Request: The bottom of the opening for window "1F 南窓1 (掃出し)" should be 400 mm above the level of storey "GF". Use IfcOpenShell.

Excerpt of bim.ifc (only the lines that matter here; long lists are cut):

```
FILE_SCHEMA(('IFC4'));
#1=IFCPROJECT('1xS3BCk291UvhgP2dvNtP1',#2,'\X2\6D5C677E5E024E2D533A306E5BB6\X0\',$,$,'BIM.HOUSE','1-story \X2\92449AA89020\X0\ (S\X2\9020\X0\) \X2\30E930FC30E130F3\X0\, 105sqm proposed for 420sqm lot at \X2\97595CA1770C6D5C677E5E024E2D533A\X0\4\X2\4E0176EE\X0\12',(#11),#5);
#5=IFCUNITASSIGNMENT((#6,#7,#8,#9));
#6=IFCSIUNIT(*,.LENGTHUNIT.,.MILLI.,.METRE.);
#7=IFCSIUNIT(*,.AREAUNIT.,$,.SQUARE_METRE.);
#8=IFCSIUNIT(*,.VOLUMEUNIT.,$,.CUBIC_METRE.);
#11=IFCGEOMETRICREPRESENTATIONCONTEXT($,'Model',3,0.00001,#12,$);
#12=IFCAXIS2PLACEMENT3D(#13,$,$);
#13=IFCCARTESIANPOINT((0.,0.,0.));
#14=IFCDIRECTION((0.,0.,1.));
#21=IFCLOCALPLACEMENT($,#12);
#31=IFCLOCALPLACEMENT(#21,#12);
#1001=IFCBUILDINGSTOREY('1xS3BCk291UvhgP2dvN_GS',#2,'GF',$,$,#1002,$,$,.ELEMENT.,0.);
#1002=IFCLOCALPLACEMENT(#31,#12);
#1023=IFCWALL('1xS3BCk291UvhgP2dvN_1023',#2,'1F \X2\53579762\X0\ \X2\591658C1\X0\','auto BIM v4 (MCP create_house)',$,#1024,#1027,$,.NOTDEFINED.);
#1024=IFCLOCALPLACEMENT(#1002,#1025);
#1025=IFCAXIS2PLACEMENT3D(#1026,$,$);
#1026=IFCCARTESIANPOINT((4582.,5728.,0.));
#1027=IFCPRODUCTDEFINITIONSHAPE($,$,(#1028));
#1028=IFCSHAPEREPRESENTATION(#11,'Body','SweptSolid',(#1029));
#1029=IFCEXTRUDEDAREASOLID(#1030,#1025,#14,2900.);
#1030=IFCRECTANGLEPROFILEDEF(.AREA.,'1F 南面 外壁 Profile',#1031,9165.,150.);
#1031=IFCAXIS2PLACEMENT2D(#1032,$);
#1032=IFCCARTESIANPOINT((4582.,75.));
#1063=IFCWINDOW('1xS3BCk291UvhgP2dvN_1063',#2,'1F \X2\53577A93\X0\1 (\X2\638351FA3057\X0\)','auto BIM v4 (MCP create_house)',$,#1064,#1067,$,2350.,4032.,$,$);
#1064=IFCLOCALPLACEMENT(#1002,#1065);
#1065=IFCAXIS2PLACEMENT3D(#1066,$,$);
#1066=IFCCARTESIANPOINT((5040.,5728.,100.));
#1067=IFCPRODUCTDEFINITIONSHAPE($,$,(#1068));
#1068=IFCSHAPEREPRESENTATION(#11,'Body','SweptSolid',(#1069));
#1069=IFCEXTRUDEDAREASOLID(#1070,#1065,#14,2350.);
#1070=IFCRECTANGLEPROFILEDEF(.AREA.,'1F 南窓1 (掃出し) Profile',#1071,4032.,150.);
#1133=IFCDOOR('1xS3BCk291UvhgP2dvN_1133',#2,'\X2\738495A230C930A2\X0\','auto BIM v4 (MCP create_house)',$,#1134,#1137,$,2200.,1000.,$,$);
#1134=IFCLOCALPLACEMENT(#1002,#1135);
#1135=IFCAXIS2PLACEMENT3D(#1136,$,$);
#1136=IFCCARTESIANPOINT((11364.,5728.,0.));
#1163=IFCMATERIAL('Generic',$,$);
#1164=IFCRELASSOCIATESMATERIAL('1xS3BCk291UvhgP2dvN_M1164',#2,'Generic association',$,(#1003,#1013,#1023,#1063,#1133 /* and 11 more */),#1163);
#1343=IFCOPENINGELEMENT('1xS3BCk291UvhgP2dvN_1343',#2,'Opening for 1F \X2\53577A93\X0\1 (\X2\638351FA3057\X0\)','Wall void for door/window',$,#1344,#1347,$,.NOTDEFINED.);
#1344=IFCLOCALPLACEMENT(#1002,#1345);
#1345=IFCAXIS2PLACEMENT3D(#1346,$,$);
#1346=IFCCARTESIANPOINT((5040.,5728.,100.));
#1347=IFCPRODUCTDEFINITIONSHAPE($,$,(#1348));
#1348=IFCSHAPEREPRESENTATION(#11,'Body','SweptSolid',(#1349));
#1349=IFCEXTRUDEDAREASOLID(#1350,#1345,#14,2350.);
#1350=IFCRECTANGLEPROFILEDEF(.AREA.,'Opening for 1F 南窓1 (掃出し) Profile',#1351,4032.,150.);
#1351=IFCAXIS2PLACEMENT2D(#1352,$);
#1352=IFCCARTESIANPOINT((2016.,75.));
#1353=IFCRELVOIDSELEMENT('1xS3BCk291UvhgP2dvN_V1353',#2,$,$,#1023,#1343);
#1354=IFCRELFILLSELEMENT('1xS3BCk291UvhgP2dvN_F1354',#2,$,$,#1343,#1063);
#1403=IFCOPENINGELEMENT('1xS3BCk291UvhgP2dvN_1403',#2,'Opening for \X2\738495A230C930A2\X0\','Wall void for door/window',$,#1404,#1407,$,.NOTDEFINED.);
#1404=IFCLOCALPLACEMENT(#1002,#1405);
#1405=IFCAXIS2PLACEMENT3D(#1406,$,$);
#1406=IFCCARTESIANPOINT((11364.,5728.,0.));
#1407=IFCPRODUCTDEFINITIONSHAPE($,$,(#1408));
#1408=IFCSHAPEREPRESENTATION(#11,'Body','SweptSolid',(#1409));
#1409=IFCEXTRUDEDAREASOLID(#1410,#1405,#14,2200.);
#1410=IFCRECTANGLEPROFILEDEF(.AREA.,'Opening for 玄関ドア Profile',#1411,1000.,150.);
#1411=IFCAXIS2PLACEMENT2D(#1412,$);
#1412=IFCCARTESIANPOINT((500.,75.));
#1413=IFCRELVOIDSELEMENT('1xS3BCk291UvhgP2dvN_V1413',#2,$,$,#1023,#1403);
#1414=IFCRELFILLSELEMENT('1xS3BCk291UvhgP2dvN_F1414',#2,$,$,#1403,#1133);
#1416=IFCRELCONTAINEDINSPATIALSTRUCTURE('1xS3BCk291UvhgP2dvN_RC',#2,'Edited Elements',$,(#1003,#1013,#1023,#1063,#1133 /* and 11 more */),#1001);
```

```python
import numpy as np
import ifcopenshell
import ifcopenshell.api.geometry
import ifcopenshell.geom
import ifcopenshell.util.element
import ifcopenshell.util.placement
import ifcopenshell.util.shape
import ifcopenshell.util.unit

model = ifcopenshell.open("bim.ifc")
unit_scale = ifcopenshell.util.unit.calculate_unit_scale(model)

window = model.by_id(1063)
opening = window.FillsVoids[0].RelatingOpeningElement
storey = ifcopenshell.util.element.get_container(window, ifc_class="IfcBuildingStorey")
level = ifcopenshell.util.placement.get_local_placement(storey.ObjectPlacement)[2, 3]

# The opening's origin need not be at the sill, so measure its lowest point.
shape = ifcopenshell.geom.create_shape(ifcopenshell.geom.settings(), opening)
bottom = ifcopenshell.util.shape.get_shape_bottom_elevation(shape, shape.geometry) / unit_scale
dz = level + 0.4 / unit_scale - bottom

shift = np.array([0.0, 0.0, dz])
# The window is not placed relative to its opening, so move both.
for product in (opening, window):
    matrix = ifcopenshell.util.placement.get_local_placement(product.ObjectPlacement)
    matrix[:3, 3] += shift
    ifcopenshell.api.geometry.edit_object_placement(model, product=product, matrix=matrix, is_si=False)

print(f"moved by {dz * unit_scale:+.3f} m")

model.write("bim-out.ifc")
```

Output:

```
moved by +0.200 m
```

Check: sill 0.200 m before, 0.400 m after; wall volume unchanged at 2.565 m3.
